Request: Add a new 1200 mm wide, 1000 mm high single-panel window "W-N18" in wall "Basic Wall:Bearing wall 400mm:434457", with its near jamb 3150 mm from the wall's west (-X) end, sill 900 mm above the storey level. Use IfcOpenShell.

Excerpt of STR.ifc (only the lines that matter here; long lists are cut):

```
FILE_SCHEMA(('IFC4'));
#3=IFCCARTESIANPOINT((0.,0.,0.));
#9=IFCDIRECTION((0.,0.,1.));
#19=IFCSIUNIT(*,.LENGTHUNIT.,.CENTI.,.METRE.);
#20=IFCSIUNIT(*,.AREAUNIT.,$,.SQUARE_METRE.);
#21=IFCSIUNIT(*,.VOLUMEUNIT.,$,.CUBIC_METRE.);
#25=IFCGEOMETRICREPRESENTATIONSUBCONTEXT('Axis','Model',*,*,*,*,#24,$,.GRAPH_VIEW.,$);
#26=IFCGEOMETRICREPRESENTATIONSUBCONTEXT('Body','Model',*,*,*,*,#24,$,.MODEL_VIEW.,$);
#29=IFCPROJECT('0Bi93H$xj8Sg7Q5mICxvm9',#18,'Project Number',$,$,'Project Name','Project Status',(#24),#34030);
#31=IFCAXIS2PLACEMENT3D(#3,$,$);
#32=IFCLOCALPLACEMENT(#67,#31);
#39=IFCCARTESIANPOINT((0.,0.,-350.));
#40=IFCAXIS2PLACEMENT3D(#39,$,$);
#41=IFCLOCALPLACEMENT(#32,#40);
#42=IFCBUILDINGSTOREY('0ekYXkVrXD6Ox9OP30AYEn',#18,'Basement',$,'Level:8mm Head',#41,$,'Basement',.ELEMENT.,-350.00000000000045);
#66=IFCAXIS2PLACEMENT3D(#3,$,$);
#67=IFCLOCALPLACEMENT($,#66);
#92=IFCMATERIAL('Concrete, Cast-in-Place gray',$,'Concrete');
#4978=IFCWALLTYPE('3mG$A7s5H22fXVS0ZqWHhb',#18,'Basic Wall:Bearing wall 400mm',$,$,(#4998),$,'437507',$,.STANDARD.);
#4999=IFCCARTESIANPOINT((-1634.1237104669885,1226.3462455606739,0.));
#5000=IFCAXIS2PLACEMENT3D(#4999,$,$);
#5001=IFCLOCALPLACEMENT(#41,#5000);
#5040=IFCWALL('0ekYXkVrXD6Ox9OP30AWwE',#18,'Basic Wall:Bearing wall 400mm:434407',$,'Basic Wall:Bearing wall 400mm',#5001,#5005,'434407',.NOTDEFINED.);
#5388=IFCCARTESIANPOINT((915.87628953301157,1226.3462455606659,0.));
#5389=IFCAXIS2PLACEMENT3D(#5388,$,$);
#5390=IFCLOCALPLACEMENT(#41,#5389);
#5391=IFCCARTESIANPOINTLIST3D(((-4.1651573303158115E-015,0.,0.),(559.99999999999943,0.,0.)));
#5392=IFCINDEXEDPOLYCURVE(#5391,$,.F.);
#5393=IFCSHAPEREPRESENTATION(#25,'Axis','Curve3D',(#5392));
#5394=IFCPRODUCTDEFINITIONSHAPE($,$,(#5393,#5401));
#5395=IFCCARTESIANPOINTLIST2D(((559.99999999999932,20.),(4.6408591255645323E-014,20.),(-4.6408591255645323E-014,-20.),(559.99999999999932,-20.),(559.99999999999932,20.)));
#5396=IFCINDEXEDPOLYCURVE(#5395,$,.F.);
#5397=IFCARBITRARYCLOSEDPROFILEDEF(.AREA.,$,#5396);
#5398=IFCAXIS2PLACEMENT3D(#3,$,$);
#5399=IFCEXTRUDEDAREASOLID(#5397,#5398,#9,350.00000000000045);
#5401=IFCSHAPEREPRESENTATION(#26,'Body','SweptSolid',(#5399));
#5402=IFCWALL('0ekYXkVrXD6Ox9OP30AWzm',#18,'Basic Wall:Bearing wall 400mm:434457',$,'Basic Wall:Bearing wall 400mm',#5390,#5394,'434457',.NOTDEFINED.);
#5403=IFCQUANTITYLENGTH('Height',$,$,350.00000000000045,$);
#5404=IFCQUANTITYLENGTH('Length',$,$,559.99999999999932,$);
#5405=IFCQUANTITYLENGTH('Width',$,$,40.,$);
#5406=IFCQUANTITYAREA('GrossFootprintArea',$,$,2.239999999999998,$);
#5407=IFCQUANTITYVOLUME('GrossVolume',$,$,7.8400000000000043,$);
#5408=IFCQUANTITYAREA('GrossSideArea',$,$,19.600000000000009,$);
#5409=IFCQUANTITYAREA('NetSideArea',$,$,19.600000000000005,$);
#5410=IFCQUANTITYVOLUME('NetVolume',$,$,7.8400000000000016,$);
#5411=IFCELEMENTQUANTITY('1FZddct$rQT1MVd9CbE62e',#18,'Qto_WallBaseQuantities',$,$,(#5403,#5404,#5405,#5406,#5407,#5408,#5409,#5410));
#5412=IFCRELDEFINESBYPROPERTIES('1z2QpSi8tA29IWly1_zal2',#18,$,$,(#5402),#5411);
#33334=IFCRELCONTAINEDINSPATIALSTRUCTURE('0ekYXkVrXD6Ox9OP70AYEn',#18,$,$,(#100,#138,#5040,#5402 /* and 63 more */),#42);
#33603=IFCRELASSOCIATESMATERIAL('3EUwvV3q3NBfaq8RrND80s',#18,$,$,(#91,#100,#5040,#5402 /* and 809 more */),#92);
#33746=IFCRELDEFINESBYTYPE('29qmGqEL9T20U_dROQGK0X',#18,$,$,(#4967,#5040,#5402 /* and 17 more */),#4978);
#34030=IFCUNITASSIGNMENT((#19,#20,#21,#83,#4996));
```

```python
import numpy as np
import ifcopenshell
import ifcopenshell.api.feature
import ifcopenshell.api.geometry
import ifcopenshell.api.pset
import ifcopenshell.api.root
import ifcopenshell.api.spatial
import ifcopenshell.geom
import ifcopenshell.util.element
import ifcopenshell.util.placement
import ifcopenshell.util.representation
import ifcopenshell.util.shape
import ifcopenshell.util.unit

model = ifcopenshell.open("STR.ifc")
unit_scale = ifcopenshell.util.unit.calculate_unit_scale(model)
area_scale = ifcopenshell.util.unit.calculate_unit_scale(model, "AREAUNIT")
volume_scale = ifcopenshell.util.unit.calculate_unit_scale(model, "VOLUMEUNIT")
settings = ifcopenshell.geom.settings()


def volume(element):
    """Net volume in cubic metres, openings subtracted."""
    shape = ifcopenshell.geom.create_shape(settings, element)
    return ifcopenshell.util.shape.get_volume(shape.geometry)


wall = model.by_guid("0ekYXkVrXD6Ox9OP30AWzm")
storey = ifcopenshell.util.element.get_container(wall, ifc_class="IfcBuildingStorey")
context = ifcopenshell.util.representation.get_context(model, "Model", "Body", "MODEL_VIEW")
before = volume(wall)

width, height, from_end, sill = 1.2, 1, 3.15, 0.9  # metres

# The wall runs along its own X axis, and the end named is its -X end.
wall_shape = ifcopenshell.geom.create_shape(settings, wall)
x, y, z = ifcopenshell.util.shape.get_vertices(wall_shape.geometry).T
start = x.min() + from_end
face, thickness = float(y.min()), float(y.max() - y.min())
wall_matrix = ifcopenshell.util.placement.get_local_placement(wall.ObjectPlacement)
level = ifcopenshell.util.placement.get_local_placement(storey.ObjectPlacement)[2, 3]


def in_wall(x, y):
    """Placement at x, y metres in the wall's axes, at sill height."""
    matrix = wall_matrix.copy()
    matrix[:, 3] = wall_matrix @ np.array([x / unit_scale, y / unit_scale, 0.0, 1.0])
    matrix[2, 3] = level + sill / unit_scale
    return matrix


# Opening: a box that overshoots both wall faces by 50 mm.
opening = ifcopenshell.api.root.create_entity(model, ifc_class="IfcOpeningElement", predefined_type="OPENING")
box = ifcopenshell.api.geometry.add_wall_representation(
    model, context=context, length=width, height=height, thickness=thickness + 0.1
)
ifcopenshell.api.geometry.assign_representation(model, product=opening, representation=box)
ifcopenshell.api.geometry.edit_object_placement(model, product=opening, matrix=in_wall(start, face - 0.05), is_si=False)
ifcopenshell.api.feature.add_feature(model, feature=opening, element=wall)

window = ifcopenshell.api.root.create_entity(model, ifc_class="IfcWindow", name="W-N18", predefined_type="WINDOW")
window.OverallWidth, window.OverallHeight = width / unit_scale, height / unit_scale
window.PartitioningType = "SINGLE_PANEL"
body = ifcopenshell.api.geometry.add_window_representation(
    model,
    context=context,
    overall_width=window.OverallWidth,
    overall_height=window.OverallHeight,
    partition_type="SINGLE_PANEL",
)
ifcopenshell.api.geometry.assign_representation(model, product=window, representation=body)
ifcopenshell.api.spatial.assign_container(model, products=[window], relating_structure=storey)
ifcopenshell.api.feature.add_filling(model, opening=opening, element=window)

# Centre the window in the wall's thickness.
ifcopenshell.api.geometry.edit_object_placement(model, product=window, matrix=in_wall(start, face), is_si=False)
window_shape = ifcopenshell.geom.create_shape(settings, window)
depth = ifcopenshell.util.shape.get_vertices(window_shape.geometry)[:, 1]
offset = face + thickness / 2 - (depth.min() + depth.max()) / 2
ifcopenshell.api.geometry.edit_object_placement(model, product=window, matrix=in_wall(start, offset), is_si=False)

after = volume(wall)

# Update the wall's stored quantities.
qto = model.by_id(ifcopenshell.util.element.get_pset(wall, "Qto_WallBaseQuantities", should_inherit=False)["id"])
ifcopenshell.api.pset.edit_qto(model, qto=qto, properties={
    "NetSideArea": after / thickness / area_scale,
    "NetVolume": after / volume_scale,
})

print(f"wall volume {before:.3f} -> {after:.3f} m3")

model.write("STR_updated.ifc")
```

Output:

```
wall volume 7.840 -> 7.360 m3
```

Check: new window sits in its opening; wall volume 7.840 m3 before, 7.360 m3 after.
